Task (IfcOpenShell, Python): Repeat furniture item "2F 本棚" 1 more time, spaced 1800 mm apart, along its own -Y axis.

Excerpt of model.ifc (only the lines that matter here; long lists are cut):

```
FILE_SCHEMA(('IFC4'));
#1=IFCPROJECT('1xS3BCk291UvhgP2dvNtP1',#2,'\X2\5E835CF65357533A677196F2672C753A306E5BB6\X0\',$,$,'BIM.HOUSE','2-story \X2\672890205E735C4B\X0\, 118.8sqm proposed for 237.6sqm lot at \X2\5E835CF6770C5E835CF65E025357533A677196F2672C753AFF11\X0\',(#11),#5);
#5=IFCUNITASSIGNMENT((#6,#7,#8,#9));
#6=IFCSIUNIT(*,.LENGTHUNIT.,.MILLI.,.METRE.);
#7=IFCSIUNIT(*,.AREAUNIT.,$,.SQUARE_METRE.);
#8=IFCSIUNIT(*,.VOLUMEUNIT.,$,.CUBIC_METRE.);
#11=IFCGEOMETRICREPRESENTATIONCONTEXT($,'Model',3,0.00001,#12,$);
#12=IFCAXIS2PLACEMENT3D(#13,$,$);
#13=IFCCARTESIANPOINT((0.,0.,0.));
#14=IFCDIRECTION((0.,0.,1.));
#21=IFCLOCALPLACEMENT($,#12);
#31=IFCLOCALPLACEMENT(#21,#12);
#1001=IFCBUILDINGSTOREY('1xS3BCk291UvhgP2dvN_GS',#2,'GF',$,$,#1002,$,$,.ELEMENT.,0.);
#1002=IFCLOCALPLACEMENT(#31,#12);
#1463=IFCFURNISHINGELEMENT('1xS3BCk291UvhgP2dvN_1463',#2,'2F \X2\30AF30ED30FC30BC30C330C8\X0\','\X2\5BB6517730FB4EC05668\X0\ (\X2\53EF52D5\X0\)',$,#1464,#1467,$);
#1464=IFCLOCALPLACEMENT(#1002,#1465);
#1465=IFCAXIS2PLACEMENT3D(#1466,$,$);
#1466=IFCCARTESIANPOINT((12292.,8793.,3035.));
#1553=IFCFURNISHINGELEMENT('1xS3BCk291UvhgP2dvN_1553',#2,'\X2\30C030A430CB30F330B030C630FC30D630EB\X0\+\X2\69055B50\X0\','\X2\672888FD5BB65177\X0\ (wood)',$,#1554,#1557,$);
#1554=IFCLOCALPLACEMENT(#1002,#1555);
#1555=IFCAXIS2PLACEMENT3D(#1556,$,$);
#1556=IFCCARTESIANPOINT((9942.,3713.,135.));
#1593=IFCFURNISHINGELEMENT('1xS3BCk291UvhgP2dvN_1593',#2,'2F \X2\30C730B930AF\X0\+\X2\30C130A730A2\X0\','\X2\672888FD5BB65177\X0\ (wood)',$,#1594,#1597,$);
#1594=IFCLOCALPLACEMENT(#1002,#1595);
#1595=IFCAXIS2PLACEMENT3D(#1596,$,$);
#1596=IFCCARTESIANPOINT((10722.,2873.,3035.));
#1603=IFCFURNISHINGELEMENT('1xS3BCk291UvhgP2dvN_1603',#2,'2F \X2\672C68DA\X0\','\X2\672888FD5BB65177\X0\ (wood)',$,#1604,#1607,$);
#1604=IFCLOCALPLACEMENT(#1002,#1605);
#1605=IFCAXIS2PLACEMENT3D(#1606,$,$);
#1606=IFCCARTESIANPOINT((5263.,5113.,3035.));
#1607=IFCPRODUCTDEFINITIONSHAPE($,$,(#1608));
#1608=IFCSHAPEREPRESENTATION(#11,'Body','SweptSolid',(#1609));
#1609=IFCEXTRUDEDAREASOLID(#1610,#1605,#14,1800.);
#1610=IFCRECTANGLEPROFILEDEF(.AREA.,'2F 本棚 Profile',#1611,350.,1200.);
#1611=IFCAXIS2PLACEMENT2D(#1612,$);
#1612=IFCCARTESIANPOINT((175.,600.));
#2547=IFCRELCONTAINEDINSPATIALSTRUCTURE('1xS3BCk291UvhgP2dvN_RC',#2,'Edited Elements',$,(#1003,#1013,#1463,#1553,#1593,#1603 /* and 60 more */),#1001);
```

```python
import ifcopenshell
import ifcopenshell.api.geometry
import ifcopenshell.api.root
import ifcopenshell.util.element
import ifcopenshell.util.placement
import ifcopenshell.util.unit

model = ifcopenshell.open("model.ifc")
unit_scale = ifcopenshell.util.unit.calculate_unit_scale(model)


def reuse_history(source, copy):
    """copy_class also copies each property set's owner history, people and application; keep the originals."""
    for rel in copy.IsDefinedBy:
        if rel.is_a("IfcRelDefinesByProperties") and (history := rel.RelatingPropertyDefinition.OwnerHistory):
            rel.RelatingPropertyDefinition.OwnerHistory = source.OwnerHistory
            ifcopenshell.util.element.remove_deep2(model, history)


source = model.by_id(1603)
base = ifcopenshell.util.placement.get_local_placement(source.ObjectPlacement)
step = -base[:3, 1] * 1.8 / unit_scale

for i in range(1, 2):
    copy = ifcopenshell.api.root.copy_class(model, product=source)
    copy.Representation = ifcopenshell.util.element.copy_deep(
        model, source.Representation, exclude=["IfcGeometricRepresentationContext", "IfcRepresentationMap"]
    )
    reuse_history(source, copy)
    matrix = base.copy()
    matrix[:3, 3] += i * step
    print("added at", matrix[:3, 3].round(3) + 0.0)
    ifcopenshell.api.geometry.edit_object_placement(model, product=copy, matrix=matrix, is_si=False)

model.write("model-out.ifc")
```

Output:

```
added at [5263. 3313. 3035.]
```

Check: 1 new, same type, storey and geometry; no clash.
